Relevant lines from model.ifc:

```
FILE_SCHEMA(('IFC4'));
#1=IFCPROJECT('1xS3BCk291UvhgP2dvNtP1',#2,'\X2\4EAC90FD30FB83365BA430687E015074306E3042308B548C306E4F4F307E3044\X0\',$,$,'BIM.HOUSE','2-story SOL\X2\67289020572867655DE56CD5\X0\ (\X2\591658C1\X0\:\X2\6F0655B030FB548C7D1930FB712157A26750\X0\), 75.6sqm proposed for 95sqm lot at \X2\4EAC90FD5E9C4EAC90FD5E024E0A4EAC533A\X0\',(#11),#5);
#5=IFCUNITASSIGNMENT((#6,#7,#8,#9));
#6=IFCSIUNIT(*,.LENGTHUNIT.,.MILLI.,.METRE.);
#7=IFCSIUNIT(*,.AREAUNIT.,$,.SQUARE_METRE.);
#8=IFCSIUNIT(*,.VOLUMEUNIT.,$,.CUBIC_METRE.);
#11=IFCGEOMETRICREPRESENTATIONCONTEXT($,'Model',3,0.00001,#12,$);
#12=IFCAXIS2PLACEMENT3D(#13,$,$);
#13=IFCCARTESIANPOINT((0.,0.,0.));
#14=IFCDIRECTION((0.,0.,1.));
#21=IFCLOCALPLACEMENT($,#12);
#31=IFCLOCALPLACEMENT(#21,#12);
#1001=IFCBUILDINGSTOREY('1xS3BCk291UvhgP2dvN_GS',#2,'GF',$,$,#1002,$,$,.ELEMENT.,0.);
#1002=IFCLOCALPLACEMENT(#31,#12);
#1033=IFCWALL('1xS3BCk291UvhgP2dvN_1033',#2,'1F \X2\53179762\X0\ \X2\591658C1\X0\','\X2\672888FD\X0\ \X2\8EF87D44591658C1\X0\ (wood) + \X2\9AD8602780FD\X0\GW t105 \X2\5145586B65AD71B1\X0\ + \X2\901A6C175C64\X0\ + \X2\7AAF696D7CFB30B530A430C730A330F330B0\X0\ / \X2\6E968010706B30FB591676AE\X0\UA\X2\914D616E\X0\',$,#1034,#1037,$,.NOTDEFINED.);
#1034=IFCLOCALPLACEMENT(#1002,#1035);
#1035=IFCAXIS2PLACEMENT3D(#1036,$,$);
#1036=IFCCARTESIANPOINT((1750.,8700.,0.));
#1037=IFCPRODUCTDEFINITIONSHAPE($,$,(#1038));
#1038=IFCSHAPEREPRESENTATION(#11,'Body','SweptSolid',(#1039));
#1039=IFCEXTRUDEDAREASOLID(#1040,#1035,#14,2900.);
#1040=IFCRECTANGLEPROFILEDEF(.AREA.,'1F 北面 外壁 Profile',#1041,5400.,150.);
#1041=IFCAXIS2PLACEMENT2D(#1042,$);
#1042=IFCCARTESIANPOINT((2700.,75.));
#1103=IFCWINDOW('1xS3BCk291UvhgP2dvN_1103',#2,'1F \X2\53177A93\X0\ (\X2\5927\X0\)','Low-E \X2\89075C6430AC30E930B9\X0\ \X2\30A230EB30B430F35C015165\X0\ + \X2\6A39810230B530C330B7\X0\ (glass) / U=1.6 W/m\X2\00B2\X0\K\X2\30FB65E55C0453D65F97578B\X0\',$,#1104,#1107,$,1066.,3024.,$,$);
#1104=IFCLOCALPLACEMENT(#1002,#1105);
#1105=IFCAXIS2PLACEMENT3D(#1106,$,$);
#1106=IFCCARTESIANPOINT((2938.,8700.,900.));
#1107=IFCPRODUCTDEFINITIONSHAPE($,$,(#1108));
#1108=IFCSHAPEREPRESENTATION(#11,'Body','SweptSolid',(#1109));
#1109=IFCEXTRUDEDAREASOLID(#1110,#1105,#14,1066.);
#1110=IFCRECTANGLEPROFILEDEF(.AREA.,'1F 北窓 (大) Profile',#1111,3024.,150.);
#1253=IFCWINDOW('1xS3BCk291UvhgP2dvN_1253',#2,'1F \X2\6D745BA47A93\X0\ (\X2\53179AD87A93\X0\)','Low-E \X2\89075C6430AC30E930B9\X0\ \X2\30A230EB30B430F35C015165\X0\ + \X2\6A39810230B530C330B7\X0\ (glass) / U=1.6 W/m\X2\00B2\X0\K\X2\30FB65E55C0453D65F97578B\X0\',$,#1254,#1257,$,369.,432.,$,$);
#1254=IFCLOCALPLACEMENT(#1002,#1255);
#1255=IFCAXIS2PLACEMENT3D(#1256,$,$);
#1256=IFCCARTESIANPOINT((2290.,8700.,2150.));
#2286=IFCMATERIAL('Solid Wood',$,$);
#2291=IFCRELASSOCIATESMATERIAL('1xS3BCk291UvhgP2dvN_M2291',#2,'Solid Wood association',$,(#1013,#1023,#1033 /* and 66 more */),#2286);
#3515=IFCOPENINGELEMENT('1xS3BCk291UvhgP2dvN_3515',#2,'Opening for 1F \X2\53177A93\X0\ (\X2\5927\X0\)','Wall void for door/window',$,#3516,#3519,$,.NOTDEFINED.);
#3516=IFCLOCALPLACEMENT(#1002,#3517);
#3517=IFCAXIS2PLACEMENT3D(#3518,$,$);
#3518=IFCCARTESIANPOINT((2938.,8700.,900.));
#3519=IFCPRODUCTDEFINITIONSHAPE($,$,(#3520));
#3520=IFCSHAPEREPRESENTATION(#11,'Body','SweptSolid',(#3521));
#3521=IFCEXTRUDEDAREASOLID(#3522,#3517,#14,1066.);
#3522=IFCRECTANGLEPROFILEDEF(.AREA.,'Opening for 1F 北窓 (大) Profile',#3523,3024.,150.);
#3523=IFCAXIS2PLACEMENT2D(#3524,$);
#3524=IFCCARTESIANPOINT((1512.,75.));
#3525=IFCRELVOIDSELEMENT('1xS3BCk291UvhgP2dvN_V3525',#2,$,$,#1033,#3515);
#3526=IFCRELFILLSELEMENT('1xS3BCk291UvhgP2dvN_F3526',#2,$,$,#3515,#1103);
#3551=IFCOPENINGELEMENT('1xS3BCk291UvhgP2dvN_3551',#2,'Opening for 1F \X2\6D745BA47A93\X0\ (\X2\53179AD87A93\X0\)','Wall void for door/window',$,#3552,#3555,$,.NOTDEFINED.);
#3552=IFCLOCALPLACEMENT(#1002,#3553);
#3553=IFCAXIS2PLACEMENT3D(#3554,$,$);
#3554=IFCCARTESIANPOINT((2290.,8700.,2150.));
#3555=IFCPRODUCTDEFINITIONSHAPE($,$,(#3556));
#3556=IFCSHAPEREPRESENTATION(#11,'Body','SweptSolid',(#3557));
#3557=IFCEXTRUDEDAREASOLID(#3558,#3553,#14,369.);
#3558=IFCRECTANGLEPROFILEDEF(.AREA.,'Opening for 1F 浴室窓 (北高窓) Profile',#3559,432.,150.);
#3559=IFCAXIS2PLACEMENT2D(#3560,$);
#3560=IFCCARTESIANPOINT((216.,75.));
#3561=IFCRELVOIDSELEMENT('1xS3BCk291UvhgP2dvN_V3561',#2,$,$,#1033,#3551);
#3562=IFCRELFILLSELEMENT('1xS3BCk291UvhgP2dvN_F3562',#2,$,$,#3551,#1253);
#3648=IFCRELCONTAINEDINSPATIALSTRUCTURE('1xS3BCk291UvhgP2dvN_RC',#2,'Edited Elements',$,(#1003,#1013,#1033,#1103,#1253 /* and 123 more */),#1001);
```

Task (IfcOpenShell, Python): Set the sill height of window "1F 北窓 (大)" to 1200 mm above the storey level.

```python
import numpy as np
import ifcopenshell
import ifcopenshell.api.geometry
import ifcopenshell.geom
import ifcopenshell.util.element
import ifcopenshell.util.placement
import ifcopenshell.util.shape
import ifcopenshell.util.unit

model = ifcopenshell.open("model.ifc")
unit_scale = ifcopenshell.util.unit.calculate_unit_scale(model)

window = model.by_guid("1xS3BCk291UvhgP2dvN_1103")
opening = window.FillsVoids[0].RelatingOpeningElement
storey = ifcopenshell.util.element.get_container(window, ifc_class="IfcBuildingStorey")
level = ifcopenshell.util.placement.get_local_placement(storey.ObjectPlacement)[2, 3]

# The opening's origin need not be at the sill, so measure its lowest point.
shape = ifcopenshell.geom.create_shape(ifcopenshell.geom.settings(), opening)
bottom = ifcopenshell.util.shape.get_shape_bottom_elevation(shape, shape.geometry) / unit_scale
dz = level + 1200.0 - bottom

shift = np.array([0.0, 0.0, dz])
# The window is not placed relative to its opening, so move both.
for product in (opening, window):
    matrix = ifcopenshell.util.placement.get_local_placement(product.ObjectPlacement)
    matrix[:3, 3] += shift
    ifcopenshell.api.geometry.edit_object_placement(model, product=product, matrix=matrix, is_si=False)

print(f"moved by {dz * unit_scale:+.3f} m")

model.write("model_rev.ifc")
```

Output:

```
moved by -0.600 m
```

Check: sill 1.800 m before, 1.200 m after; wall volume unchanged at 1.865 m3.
